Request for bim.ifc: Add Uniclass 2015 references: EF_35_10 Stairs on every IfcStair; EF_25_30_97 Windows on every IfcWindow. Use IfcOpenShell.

First a look at what the model holds.

```python
import ifcopenshell

model = ifcopenshell.open("bim.ifc")
print(model.schema)
print("classifications:", [c.Name for c in model.by_type("IfcClassification")])
for ifc_class in ("IfcDoor", "IfcRoof", "IfcStair", "IfcWall", "IfcWindow"):
    print(ifc_class, len(model.by_type(ifc_class)))
```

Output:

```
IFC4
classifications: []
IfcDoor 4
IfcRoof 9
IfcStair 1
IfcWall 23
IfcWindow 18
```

```python
import ifcopenshell
import ifcopenshell.api.classification

model = ifcopenshell.open("bim.ifc")

system = ifcopenshell.api.classification.add_classification(model, classification="Uniclass 2015")

codes = {
    "IfcStair": ("EF_35_10", "Stairs"),
    "IfcWindow": ("EF_25_30_97", "Windows"),
}
for ifc_class, (code, name) in codes.items():
    products = model.by_type(ifc_class)
    ifcopenshell.api.classification.add_reference(
        model, products=products, classification=system, identification=code, name=name
    )
    print(code, len(products))

model.write("bim_updated.ifc")
```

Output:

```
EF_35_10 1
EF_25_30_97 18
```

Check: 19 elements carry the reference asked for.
